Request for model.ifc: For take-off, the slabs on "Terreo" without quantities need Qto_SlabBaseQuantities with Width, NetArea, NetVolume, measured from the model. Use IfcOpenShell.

First a look at what the model holds.

```python
import ifcopenshell
import ifcopenshell.util.element
import ifcopenshell.util.unit

model = ifcopenshell.open("model.ifc")
print(model.schema)
for unit_type in ("LENGTHUNIT", "AREAUNIT", "VOLUMEUNIT"):
    print(unit_type, ifcopenshell.util.unit.calculate_unit_scale(model, unit_type))
storey = next(s for s in model.by_type("IfcBuildingStorey") if s.Name == "Terreo")
slabs = [e for e in ifcopenshell.util.element.get_decomposition(storey) if e.is_a("IfcSlab")]
for e in sorted(slabs, key=lambda e: e.id()):
    print(e.id(), e.is_a(), e.Name, list(ifcopenshell.util.element.get_psets(e, qtos_only=True)), sep=" | ")
```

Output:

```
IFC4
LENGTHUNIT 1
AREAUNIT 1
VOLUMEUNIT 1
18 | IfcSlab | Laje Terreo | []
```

```python
import ifcopenshell
import ifcopenshell.api.pset
import ifcopenshell.geom
import ifcopenshell.util.element
import ifcopenshell.util.shape
import ifcopenshell.util.unit

model = ifcopenshell.open("model.ifc")
unit_scale = ifcopenshell.util.unit.calculate_unit_scale(model)
area_scale = ifcopenshell.util.unit.calculate_unit_scale(model, "AREAUNIT")
volume_scale = ifcopenshell.util.unit.calculate_unit_scale(model, "VOLUMEUNIT")
settings = ifcopenshell.geom.settings()

storey = next(s for s in model.by_type("IfcBuildingStorey") if s.Name == "Terreo")
slabs = [e for e in ifcopenshell.util.element.get_decomposition(storey) if e.is_a("IfcSlab")]

for e in sorted(slabs, key=lambda e: e.id()):
    if ifcopenshell.util.element.get_psets(e, qtos_only=True, should_inherit=False):
        continue
    # Geometry comes back in metres, in the element's own axes.
    shape = ifcopenshell.geom.create_shape(settings, e)
    values = {
        "Width": ifcopenshell.util.shape.get_z(shape.geometry) / unit_scale,
        "NetArea": ifcopenshell.util.shape.get_footprint_area(shape.geometry) / area_scale,
        "NetVolume": ifcopenshell.util.shape.get_volume(shape.geometry) / volume_scale,
    }
    qto = ifcopenshell.api.pset.add_qto(model, product=e, name="Qto_SlabBaseQuantities")
    ifcopenshell.api.pset.edit_qto(model, qto=qto, properties=values)
    print(e.id(), {k: round(v, 3) for k, v in values.items()})

model.write("model_updated.ifc")
```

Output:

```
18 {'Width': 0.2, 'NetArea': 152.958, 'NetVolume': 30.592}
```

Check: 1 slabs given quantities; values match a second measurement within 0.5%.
